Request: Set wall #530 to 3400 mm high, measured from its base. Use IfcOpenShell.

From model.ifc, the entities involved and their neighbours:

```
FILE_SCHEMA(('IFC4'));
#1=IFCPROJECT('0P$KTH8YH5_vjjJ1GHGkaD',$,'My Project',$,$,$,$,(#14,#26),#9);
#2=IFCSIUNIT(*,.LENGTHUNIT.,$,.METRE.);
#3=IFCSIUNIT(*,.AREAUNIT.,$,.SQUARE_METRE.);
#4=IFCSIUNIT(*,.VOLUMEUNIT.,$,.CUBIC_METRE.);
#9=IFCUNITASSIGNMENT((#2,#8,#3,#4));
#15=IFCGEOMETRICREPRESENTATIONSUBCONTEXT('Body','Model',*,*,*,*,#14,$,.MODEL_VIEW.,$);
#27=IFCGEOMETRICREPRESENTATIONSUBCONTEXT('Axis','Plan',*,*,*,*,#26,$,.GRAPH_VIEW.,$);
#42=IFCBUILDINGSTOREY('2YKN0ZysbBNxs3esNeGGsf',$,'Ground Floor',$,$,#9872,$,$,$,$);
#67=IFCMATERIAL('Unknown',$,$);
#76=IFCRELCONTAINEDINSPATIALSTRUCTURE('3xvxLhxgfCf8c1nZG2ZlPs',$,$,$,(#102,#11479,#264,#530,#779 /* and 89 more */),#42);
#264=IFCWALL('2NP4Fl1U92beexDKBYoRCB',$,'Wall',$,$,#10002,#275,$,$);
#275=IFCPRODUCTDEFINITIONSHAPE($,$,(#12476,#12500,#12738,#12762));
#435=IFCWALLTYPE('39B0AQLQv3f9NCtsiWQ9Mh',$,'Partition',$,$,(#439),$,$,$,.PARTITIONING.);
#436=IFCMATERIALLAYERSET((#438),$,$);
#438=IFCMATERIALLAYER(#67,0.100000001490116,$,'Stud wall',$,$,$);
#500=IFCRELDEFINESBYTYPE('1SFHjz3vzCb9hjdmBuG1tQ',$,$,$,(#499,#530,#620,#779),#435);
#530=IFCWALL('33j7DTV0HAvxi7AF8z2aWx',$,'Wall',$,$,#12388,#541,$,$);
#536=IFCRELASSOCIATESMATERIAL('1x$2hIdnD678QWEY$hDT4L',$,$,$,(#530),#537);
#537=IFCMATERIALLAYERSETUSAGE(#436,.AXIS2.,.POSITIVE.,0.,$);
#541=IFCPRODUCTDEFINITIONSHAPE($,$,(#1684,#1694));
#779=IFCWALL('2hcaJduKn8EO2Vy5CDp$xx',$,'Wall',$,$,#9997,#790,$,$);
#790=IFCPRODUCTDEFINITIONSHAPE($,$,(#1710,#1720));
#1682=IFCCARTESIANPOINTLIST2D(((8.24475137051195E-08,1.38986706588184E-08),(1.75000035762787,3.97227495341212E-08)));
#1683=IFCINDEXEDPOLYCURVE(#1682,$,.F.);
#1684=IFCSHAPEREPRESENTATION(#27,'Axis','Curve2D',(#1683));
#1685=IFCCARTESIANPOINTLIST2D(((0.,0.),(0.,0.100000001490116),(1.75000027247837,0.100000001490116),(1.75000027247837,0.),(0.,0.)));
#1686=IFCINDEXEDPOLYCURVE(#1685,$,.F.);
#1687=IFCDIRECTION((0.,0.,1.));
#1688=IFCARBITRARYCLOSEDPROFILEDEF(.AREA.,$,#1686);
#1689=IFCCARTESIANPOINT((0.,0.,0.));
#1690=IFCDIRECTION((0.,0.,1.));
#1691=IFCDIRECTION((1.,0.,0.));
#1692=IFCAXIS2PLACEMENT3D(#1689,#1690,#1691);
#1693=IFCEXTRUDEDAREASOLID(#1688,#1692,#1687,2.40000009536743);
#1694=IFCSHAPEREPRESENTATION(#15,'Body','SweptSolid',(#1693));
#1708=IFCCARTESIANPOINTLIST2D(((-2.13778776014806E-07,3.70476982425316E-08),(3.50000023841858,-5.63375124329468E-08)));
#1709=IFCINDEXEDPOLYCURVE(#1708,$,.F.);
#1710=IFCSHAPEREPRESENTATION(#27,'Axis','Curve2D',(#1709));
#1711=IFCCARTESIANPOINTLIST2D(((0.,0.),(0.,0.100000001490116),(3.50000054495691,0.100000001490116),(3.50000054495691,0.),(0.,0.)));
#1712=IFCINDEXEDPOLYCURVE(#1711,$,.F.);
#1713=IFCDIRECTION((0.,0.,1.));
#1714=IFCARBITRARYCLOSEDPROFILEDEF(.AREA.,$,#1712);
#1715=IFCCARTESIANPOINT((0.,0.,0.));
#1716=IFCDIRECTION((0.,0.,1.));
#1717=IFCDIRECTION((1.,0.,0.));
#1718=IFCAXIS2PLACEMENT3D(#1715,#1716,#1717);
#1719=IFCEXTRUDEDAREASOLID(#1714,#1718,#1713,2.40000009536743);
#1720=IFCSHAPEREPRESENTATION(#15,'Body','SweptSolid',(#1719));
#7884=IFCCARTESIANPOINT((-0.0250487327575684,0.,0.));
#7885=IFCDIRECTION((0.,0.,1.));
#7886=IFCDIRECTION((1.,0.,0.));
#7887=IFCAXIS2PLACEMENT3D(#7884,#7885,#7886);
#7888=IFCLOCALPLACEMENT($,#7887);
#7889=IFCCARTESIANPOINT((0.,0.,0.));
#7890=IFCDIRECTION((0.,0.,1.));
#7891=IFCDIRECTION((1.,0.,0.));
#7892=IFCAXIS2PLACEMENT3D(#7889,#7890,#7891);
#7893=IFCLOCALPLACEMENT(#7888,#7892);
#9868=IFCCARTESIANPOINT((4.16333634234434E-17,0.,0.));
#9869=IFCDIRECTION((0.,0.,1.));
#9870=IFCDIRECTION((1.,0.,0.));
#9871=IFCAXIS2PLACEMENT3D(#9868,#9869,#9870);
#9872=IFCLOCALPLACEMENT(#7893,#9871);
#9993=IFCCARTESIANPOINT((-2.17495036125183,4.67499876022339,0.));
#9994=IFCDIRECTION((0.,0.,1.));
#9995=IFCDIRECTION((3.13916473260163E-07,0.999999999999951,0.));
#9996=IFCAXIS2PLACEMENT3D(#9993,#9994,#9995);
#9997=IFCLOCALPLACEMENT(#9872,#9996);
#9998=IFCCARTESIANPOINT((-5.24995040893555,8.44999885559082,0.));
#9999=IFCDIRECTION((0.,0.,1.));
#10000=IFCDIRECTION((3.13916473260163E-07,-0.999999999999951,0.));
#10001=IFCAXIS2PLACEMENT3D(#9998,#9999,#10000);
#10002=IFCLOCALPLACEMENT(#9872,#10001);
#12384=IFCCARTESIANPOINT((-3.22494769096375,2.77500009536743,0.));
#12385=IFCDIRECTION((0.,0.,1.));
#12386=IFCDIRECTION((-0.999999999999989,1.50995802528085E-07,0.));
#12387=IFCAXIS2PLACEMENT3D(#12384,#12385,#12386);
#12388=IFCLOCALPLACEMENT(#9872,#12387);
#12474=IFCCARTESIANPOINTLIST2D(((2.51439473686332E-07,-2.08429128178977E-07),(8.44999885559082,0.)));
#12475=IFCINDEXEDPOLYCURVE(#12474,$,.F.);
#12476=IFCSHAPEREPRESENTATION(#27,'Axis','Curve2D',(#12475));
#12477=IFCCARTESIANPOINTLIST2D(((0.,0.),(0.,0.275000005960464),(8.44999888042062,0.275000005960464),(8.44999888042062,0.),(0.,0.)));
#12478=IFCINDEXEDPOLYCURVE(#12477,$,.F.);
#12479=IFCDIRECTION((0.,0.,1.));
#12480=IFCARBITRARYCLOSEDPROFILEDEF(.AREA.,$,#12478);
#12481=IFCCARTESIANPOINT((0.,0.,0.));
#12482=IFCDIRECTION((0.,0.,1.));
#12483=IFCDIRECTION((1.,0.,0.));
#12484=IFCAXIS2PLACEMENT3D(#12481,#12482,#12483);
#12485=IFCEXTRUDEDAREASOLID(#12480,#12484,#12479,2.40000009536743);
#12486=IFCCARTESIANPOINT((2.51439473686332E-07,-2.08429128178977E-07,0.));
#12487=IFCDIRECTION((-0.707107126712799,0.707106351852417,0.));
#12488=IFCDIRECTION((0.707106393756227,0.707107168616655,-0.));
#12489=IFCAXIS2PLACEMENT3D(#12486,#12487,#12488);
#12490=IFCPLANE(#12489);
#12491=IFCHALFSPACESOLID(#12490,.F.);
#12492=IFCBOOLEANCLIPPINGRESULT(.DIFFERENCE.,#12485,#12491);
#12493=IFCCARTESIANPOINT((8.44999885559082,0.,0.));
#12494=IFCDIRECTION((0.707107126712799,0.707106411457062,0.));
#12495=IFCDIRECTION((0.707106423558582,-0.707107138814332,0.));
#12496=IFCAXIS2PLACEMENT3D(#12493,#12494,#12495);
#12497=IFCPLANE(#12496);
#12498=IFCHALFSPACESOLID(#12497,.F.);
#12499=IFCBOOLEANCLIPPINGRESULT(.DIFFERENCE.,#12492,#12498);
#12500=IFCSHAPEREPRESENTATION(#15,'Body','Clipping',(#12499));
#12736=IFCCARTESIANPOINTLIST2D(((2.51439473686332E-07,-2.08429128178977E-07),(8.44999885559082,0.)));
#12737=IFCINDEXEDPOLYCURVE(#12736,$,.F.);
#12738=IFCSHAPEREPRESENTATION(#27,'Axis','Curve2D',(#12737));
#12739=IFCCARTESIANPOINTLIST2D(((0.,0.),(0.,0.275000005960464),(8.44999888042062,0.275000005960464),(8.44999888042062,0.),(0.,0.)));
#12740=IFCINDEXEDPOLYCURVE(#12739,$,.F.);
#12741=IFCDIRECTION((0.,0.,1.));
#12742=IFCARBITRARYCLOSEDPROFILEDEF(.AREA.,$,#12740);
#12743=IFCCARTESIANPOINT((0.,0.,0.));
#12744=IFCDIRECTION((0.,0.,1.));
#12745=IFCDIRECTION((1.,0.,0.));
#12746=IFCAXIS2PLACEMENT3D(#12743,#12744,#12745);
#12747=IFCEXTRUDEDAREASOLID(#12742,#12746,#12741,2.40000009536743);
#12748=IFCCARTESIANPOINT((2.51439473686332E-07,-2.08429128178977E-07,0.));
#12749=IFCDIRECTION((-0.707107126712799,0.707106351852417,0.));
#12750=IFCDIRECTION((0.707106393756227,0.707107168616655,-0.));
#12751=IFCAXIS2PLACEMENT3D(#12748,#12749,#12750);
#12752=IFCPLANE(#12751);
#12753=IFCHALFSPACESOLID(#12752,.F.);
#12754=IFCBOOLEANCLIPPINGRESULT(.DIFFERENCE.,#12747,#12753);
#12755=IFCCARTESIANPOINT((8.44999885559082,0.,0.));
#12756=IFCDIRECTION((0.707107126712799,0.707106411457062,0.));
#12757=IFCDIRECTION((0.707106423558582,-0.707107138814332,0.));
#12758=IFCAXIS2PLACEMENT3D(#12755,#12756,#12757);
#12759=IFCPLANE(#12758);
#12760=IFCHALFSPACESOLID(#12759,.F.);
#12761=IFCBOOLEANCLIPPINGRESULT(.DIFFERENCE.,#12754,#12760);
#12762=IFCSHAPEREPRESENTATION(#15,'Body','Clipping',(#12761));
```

```python
import ifcopenshell
import ifcopenshell.geom
import ifcopenshell.util.representation
import ifcopenshell.util.shape
import ifcopenshell.util.unit

model = ifcopenshell.open("model.ifc")
unit_scale = ifcopenshell.util.unit.calculate_unit_scale(model)
settings = ifcopenshell.geom.settings()


def volume(element):
    """Net volume in cubic metres, openings subtracted."""
    shape = ifcopenshell.geom.create_shape(settings, element)
    return ifcopenshell.util.shape.get_volume(shape.geometry)


wall = model.by_guid("33j7DTV0HAvxi7AF8z2aWx")
before = volume(wall)

body = ifcopenshell.util.representation.get_representation(wall, "Model", "Body")
solid = body.Items[0]
old_height = solid.Depth
solid.Depth = 3.4 / unit_scale
after = volume(wall)

print(f"height {old_height:g} -> {solid.Depth:g}, volume {before:.3f} -> {after:.3f} m3")

model.write("model_updated.ifc")
```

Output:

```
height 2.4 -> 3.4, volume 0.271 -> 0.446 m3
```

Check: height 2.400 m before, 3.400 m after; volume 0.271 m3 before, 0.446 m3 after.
